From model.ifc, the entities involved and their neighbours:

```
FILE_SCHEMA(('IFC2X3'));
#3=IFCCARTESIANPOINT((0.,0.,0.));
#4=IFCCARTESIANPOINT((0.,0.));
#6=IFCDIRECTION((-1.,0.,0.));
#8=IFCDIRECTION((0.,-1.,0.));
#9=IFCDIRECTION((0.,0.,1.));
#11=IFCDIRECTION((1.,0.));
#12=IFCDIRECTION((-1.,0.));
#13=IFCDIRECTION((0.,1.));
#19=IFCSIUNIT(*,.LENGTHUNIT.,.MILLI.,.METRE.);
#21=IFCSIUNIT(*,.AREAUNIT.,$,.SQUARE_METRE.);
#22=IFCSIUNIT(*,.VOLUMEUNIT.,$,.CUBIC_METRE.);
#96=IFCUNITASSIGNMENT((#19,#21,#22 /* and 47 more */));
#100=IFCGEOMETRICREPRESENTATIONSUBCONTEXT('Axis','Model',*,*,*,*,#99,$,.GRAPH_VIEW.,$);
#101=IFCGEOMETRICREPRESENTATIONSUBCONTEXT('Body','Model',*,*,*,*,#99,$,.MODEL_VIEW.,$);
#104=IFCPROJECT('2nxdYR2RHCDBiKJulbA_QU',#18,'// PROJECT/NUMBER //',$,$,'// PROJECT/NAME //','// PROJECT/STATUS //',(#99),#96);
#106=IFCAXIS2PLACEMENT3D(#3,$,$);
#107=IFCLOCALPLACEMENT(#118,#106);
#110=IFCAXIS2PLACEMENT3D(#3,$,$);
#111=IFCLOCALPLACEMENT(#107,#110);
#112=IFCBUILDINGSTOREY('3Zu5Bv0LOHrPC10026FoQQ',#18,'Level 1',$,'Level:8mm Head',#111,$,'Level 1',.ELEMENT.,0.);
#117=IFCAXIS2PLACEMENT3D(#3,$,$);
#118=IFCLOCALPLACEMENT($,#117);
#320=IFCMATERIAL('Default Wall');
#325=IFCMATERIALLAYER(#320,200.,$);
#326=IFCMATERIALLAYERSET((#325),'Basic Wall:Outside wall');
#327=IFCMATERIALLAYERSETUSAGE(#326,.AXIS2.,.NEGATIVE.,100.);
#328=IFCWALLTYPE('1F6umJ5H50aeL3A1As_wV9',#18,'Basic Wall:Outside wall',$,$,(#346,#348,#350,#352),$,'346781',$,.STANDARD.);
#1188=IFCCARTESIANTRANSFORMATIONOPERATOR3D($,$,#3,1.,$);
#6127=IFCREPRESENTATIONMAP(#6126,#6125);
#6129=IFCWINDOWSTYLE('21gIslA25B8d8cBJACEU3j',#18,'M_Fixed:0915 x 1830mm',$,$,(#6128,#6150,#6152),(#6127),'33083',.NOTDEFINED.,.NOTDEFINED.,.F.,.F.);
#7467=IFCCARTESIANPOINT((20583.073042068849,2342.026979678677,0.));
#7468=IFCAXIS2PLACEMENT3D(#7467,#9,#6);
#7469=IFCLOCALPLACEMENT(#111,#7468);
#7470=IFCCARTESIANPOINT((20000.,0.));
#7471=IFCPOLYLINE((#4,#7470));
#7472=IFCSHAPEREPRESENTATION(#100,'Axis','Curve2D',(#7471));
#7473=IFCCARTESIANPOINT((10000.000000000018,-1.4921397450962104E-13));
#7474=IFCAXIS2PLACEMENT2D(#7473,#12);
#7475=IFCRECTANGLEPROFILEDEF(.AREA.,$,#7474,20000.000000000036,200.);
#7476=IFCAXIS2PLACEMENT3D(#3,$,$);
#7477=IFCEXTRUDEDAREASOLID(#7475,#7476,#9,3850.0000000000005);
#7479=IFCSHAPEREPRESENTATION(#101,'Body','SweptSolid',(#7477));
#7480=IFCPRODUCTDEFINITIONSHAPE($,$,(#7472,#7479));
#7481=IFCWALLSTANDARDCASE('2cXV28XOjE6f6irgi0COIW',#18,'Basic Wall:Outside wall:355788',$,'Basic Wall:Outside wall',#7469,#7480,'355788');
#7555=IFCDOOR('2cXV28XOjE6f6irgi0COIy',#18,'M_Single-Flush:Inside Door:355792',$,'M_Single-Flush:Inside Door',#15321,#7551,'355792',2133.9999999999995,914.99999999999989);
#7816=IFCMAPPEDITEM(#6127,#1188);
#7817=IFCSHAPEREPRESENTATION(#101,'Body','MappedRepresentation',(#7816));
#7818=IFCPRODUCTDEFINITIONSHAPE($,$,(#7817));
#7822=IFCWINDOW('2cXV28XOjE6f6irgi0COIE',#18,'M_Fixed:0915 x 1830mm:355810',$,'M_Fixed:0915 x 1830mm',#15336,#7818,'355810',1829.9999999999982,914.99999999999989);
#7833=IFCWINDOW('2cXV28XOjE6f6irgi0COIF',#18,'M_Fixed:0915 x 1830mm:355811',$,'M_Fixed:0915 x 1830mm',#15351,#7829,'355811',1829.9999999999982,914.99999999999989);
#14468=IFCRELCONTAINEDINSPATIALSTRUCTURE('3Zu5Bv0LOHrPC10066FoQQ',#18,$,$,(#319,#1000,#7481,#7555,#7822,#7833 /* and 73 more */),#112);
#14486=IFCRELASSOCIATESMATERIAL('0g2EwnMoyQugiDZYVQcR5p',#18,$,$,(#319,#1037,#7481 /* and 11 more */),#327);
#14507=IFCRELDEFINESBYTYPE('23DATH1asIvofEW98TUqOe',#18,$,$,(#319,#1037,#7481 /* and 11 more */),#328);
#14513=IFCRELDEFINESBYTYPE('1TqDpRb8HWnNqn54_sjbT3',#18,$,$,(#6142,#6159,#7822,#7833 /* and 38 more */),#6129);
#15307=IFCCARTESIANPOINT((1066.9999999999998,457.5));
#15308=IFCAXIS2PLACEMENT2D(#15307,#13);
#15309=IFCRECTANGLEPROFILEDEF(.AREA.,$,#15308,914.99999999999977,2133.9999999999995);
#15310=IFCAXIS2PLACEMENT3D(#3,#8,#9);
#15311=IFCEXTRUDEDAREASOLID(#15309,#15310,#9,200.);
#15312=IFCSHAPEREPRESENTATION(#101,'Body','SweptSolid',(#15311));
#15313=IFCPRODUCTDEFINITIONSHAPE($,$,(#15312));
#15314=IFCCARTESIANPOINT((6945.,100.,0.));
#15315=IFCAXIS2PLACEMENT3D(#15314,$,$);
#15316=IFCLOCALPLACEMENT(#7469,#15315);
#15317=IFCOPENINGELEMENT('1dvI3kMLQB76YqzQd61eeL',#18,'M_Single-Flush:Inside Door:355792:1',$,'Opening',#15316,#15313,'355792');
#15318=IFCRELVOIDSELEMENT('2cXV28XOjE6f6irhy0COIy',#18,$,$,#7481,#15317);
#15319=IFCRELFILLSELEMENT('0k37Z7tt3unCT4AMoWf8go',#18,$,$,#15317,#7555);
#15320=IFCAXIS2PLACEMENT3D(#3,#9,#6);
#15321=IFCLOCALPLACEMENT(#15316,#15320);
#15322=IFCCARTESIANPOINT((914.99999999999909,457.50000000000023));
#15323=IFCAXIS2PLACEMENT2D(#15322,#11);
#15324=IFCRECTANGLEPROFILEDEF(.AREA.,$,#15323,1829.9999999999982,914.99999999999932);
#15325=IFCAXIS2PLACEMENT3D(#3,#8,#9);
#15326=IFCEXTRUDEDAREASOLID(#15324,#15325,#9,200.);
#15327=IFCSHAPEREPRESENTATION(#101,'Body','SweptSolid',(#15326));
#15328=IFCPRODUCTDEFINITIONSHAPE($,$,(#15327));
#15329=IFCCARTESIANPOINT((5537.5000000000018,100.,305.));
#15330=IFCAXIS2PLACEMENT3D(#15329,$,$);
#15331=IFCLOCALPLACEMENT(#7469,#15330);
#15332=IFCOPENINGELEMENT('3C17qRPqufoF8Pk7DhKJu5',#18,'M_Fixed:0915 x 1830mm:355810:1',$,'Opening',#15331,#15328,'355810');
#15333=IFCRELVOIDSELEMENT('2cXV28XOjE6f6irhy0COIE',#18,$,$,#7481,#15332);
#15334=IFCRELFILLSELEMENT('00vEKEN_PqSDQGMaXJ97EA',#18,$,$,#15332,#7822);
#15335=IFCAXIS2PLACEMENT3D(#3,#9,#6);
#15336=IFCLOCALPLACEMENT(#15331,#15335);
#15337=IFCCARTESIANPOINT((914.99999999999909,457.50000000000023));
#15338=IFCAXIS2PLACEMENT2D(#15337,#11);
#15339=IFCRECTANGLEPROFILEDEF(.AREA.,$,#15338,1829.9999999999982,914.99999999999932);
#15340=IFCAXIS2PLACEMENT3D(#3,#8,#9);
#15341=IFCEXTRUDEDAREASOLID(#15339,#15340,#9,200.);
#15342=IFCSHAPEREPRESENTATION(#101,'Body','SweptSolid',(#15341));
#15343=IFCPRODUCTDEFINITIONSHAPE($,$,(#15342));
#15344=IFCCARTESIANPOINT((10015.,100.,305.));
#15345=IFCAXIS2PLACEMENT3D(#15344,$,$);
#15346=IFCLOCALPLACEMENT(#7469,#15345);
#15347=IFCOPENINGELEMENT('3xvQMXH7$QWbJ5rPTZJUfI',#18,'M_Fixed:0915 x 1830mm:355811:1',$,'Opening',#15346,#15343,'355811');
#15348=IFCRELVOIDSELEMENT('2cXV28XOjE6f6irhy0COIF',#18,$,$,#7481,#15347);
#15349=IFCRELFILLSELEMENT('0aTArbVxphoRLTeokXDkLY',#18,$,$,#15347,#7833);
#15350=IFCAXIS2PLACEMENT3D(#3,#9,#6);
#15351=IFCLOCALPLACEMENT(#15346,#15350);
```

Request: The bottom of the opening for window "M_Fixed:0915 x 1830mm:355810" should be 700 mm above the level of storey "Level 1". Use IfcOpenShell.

```python
import numpy as np
import ifcopenshell
import ifcopenshell.api.geometry
import ifcopenshell.geom
import ifcopenshell.util.element
import ifcopenshell.util.placement
import ifcopenshell.util.shape
import ifcopenshell.util.unit

model = ifcopenshell.open("model.ifc")
unit_scale = ifcopenshell.util.unit.calculate_unit_scale(model)

window = model.by_guid("2cXV28XOjE6f6irgi0COIE")
opening = window.FillsVoids[0].RelatingOpeningElement
storey = ifcopenshell.util.element.get_container(window, ifc_class="IfcBuildingStorey")
level = ifcopenshell.util.placement.get_local_placement(storey.ObjectPlacement)[2, 3]

# The opening's origin need not be at the sill, so measure its lowest point.
shape = ifcopenshell.geom.create_shape(ifcopenshell.geom.settings(), opening)
bottom = ifcopenshell.util.shape.get_shape_bottom_elevation(shape, shape.geometry) / unit_scale
dz = level + 700.0 - bottom

shift = np.array([0.0, 0.0, dz])
# The window is placed relative to its opening, so it follows when the opening moves.
matrix = ifcopenshell.util.placement.get_local_placement(opening.ObjectPlacement)
matrix[:3, 3] += shift
ifcopenshell.api.geometry.edit_object_placement(
    model, product=opening, matrix=matrix, is_si=False, should_transform_children=True
)

print(f"moved by {dz * unit_scale:+.3f} m")

model.write("model_rev.ifc")
```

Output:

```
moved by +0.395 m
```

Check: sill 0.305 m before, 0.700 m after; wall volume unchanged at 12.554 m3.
